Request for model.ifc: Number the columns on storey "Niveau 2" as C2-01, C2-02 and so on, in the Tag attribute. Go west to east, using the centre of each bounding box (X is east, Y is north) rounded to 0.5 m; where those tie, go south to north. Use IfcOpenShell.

First a look at what the model holds.

```python
import ifcopenshell
import ifcopenshell.util.element
import ifcopenshell.util.placement

model = ifcopenshell.open("model.ifc")
print(model.schema)
storey = next(s for s in model.by_type("IfcBuildingStorey") if s.Name == "Niveau 2")
columns = [e for e in ifcopenshell.util.element.get_decomposition(storey) if e.is_a("IfcColumn")]
for e in sorted(columns, key=lambda e: e.id()):
    origin = ifcopenshell.util.placement.get_local_placement(e.ObjectPlacement)[:3, 3]
    print(e.id(), e.Tag, e.Name, origin.round(2) + 0.0, sep=" | ")
```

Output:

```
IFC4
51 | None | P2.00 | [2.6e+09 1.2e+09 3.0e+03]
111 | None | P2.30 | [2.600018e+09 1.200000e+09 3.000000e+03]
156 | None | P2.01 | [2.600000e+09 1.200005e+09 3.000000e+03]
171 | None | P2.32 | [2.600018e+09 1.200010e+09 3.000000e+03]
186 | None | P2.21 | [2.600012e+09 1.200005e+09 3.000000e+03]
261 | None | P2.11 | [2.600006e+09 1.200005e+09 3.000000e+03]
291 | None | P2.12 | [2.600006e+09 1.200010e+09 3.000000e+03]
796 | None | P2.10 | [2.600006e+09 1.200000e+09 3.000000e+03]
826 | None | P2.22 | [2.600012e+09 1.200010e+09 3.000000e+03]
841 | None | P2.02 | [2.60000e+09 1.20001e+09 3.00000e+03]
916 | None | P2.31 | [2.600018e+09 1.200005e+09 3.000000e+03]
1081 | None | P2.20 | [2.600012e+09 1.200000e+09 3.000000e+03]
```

```python
import ifcopenshell
import ifcopenshell.geom
import ifcopenshell.util.element
import ifcopenshell.util.shape

model = ifcopenshell.open("model.ifc")
settings = ifcopenshell.geom.settings()
settings.set("use-world-coords", True)


def centre(element):
    shape = ifcopenshell.geom.create_shape(settings, element)
    return ifcopenshell.util.shape.get_bbox_centroid(shape.geometry)


storey = next(s for s in model.by_type("IfcBuildingStorey") if s.Name == "Niveau 2")
columns = [e for e in ifcopenshell.util.element.get_decomposition(storey) if e.is_a("IfcColumn")]

# Insertion points can sit at a corner or the storey origin, so sort by the geometry (in metres).
centres = {e: centre(e) for e in columns}
columns.sort(key=lambda e: (round(centres[e][0] / 0.5), centres[e][1]))

for i, e in enumerate(columns, start=1):
    number = f"C2-{i:02d}"
    e.Tag = number
    print(e.id(), number)

model.write("model_v2.ifc")
```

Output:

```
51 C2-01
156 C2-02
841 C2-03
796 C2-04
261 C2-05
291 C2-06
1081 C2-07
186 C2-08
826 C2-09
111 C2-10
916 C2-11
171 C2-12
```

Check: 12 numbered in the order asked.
